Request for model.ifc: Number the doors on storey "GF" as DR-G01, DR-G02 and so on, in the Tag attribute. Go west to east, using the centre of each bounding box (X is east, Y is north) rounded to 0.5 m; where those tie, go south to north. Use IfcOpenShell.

First a look at what the model holds.

```python
import ifcopenshell
import ifcopenshell.util.element
import ifcopenshell.util.placement

model = ifcopenshell.open("model.ifc")
print(model.schema)
storey = next(s for s in model.by_type("IfcBuildingStorey") if s.Name == "GF")
doors = [e for e in ifcopenshell.util.element.get_decomposition(storey) if e.is_a("IfcDoor")]
for e in sorted(doors, key=lambda e: e.id()):
    origin = ifcopenshell.util.placement.get_local_placement(e.ObjectPlacement)[:3, 3]
    print(e.id(), e.Tag, e.Name, origin.round(2) + 0.0, sep=" | ")
```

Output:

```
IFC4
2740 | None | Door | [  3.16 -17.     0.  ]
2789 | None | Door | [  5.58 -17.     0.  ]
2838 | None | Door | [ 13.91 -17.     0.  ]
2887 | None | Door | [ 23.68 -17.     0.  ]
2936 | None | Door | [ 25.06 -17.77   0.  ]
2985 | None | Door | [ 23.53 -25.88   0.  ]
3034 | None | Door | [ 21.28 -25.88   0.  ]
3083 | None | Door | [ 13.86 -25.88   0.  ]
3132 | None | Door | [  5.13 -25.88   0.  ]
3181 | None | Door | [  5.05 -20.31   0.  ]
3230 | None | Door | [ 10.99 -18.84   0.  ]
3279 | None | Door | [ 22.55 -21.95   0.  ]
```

```python
import ifcopenshell
import ifcopenshell.geom
import ifcopenshell.util.element
import ifcopenshell.util.shape

model = ifcopenshell.open("model.ifc")
settings = ifcopenshell.geom.settings()
settings.set("use-world-coords", True)


def centre(element):
    shape = ifcopenshell.geom.create_shape(settings, element)
    return ifcopenshell.util.shape.get_bbox_centroid(shape.geometry)


storey = next(s for s in model.by_type("IfcBuildingStorey") if s.Name == "GF")
doors = [e for e in ifcopenshell.util.element.get_decomposition(storey) if e.is_a("IfcDoor")]

# Insertion points can sit at a corner or the storey origin, so sort by the geometry (in metres).
centres = {e: centre(e) for e in doors}
doors.sort(key=lambda e: (round(centres[e][0] / 0.5), centres[e][1]))

for i, e in enumerate(doors, start=1):
    number = f"DR-G{i:02d}"
    e.Tag = number
    print(e.id(), number)

model.write("model_rev.ifc")
```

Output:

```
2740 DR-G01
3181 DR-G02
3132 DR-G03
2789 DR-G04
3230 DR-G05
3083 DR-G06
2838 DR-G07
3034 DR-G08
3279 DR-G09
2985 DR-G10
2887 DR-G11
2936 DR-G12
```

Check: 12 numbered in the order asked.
